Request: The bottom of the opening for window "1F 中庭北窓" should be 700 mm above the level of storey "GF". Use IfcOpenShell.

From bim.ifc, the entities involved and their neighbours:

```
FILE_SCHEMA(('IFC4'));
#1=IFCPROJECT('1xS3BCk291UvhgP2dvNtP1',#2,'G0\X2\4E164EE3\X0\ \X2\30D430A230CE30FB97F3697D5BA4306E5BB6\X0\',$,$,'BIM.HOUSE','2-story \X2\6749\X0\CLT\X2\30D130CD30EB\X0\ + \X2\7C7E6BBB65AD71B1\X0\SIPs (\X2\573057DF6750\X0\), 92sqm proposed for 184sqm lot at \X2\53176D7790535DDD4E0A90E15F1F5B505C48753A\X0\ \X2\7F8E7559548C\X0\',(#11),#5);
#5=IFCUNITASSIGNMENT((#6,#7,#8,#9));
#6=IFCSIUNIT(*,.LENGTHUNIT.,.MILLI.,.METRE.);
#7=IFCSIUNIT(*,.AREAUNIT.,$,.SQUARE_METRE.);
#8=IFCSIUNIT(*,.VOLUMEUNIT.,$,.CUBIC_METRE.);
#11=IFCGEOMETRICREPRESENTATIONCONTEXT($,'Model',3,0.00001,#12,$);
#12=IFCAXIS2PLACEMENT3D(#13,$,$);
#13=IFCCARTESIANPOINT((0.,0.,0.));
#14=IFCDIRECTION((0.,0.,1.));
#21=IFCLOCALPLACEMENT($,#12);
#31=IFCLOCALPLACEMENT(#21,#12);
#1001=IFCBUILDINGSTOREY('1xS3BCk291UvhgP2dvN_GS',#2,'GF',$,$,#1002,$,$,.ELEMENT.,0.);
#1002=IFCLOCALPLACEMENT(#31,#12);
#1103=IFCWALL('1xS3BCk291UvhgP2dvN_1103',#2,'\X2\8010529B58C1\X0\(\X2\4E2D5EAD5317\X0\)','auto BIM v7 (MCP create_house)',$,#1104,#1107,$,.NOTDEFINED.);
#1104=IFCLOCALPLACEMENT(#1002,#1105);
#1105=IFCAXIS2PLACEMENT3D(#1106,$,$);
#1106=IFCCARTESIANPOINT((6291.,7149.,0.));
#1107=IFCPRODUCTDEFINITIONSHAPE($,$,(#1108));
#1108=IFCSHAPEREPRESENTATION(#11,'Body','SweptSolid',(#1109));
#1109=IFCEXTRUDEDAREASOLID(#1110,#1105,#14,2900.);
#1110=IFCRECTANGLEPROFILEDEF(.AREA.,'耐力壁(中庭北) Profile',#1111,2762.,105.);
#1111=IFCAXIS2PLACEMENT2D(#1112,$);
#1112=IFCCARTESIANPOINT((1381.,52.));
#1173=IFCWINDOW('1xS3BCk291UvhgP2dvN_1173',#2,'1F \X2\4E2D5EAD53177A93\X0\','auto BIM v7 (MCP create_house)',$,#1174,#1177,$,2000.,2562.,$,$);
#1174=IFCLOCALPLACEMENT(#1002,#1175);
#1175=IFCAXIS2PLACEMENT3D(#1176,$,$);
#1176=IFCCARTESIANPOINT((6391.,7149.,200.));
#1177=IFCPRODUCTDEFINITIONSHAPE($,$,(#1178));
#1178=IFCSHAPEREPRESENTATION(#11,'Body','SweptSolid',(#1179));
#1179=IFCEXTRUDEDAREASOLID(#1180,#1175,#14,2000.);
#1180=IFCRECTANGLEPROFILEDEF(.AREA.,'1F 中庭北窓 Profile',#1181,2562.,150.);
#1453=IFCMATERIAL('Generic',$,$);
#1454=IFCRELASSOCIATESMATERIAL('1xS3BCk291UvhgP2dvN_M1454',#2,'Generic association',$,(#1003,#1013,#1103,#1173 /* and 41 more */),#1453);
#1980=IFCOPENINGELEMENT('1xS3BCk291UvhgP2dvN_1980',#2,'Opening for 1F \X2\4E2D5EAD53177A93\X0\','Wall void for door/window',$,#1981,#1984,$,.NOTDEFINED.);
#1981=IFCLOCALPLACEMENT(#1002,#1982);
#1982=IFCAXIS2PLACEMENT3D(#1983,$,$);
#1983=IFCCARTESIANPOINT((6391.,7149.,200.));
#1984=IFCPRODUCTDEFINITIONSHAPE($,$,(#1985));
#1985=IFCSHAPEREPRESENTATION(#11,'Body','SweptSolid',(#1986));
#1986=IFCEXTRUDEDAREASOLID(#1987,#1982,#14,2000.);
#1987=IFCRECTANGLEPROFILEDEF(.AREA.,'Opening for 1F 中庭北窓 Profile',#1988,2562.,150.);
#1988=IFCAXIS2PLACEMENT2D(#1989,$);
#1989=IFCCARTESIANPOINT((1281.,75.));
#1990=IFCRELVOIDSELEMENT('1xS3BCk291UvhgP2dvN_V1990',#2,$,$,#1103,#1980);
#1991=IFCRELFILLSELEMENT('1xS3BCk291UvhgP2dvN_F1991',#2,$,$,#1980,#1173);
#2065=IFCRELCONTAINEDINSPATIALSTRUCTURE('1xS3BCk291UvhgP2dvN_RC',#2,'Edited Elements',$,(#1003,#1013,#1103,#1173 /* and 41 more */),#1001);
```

```python
import numpy as np
import ifcopenshell
import ifcopenshell.api.geometry
import ifcopenshell.geom
import ifcopenshell.util.element
import ifcopenshell.util.placement
import ifcopenshell.util.shape
import ifcopenshell.util.unit

model = ifcopenshell.open("bim.ifc")
unit_scale = ifcopenshell.util.unit.calculate_unit_scale(model)

window = model.by_guid("1xS3BCk291UvhgP2dvN_1173")
opening = window.FillsVoids[0].RelatingOpeningElement
storey = ifcopenshell.util.element.get_container(window, ifc_class="IfcBuildingStorey")
level = ifcopenshell.util.placement.get_local_placement(storey.ObjectPlacement)[2, 3]

# The opening's origin need not be at the sill, so measure its lowest point.
shape = ifcopenshell.geom.create_shape(ifcopenshell.geom.settings(), opening)
bottom = ifcopenshell.util.shape.get_shape_bottom_elevation(shape, shape.geometry) / unit_scale
dz = level + 0.7 / unit_scale - bottom

shift = np.array([0.0, 0.0, dz])
# The window is not placed relative to its opening, so move both.
for product in (opening, window):
    matrix = ifcopenshell.util.placement.get_local_placement(product.ObjectPlacement)
    matrix[:3, 3] += shift
    ifcopenshell.api.geometry.edit_object_placement(model, product=product, matrix=matrix, is_si=False)

print(f"moved by {dz * unit_scale:+.3f} m")

model.write("bim_edited.ifc")
```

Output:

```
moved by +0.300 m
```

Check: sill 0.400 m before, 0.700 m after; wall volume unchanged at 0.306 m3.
